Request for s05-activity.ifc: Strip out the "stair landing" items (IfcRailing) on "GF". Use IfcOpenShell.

First a look at what the model holds.

```python
import ifcopenshell
import ifcopenshell.util.element

model = ifcopenshell.open("s05-activity.ifc")
print(model.schema)
storey = next(s for s in model.by_type("IfcBuildingStorey") if s.Name == "GF")
railings = [e for e in ifcopenshell.util.element.get_decomposition(storey) if e.is_a("IfcRailing")]
seen = {}
for e in railings:
    element_type = ifcopenshell.util.element.get_type(e)
    name = element_type.Name if element_type not in (None, e) else None
    seen[name] = seen.get(name, 0) + 1
for name, count in sorted(seen.items(), key=str):
    print(count, "x", name)
```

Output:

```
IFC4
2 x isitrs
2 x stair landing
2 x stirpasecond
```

```python
import ifcopenshell
import ifcopenshell.api.root
import ifcopenshell.util.element

model = ifcopenshell.open("s05-activity.ifc")

storey = next(s for s in model.by_type("IfcBuildingStorey") if s.Name == "GF")
railings = [e for e in ifcopenshell.util.element.get_decomposition(storey) if e.is_a("IfcRailing")]
targets = [e for e in railings if (t := ifcopenshell.util.element.get_type(e)) not in (None, e) and t.Name == "stair landing"]

for e in targets:
    ifcopenshell.api.root.remove_product(model, product=e)
print(len(targets), "removed")

model.write("s05-activity_v2.ifc")
```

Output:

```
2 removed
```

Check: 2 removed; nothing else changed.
